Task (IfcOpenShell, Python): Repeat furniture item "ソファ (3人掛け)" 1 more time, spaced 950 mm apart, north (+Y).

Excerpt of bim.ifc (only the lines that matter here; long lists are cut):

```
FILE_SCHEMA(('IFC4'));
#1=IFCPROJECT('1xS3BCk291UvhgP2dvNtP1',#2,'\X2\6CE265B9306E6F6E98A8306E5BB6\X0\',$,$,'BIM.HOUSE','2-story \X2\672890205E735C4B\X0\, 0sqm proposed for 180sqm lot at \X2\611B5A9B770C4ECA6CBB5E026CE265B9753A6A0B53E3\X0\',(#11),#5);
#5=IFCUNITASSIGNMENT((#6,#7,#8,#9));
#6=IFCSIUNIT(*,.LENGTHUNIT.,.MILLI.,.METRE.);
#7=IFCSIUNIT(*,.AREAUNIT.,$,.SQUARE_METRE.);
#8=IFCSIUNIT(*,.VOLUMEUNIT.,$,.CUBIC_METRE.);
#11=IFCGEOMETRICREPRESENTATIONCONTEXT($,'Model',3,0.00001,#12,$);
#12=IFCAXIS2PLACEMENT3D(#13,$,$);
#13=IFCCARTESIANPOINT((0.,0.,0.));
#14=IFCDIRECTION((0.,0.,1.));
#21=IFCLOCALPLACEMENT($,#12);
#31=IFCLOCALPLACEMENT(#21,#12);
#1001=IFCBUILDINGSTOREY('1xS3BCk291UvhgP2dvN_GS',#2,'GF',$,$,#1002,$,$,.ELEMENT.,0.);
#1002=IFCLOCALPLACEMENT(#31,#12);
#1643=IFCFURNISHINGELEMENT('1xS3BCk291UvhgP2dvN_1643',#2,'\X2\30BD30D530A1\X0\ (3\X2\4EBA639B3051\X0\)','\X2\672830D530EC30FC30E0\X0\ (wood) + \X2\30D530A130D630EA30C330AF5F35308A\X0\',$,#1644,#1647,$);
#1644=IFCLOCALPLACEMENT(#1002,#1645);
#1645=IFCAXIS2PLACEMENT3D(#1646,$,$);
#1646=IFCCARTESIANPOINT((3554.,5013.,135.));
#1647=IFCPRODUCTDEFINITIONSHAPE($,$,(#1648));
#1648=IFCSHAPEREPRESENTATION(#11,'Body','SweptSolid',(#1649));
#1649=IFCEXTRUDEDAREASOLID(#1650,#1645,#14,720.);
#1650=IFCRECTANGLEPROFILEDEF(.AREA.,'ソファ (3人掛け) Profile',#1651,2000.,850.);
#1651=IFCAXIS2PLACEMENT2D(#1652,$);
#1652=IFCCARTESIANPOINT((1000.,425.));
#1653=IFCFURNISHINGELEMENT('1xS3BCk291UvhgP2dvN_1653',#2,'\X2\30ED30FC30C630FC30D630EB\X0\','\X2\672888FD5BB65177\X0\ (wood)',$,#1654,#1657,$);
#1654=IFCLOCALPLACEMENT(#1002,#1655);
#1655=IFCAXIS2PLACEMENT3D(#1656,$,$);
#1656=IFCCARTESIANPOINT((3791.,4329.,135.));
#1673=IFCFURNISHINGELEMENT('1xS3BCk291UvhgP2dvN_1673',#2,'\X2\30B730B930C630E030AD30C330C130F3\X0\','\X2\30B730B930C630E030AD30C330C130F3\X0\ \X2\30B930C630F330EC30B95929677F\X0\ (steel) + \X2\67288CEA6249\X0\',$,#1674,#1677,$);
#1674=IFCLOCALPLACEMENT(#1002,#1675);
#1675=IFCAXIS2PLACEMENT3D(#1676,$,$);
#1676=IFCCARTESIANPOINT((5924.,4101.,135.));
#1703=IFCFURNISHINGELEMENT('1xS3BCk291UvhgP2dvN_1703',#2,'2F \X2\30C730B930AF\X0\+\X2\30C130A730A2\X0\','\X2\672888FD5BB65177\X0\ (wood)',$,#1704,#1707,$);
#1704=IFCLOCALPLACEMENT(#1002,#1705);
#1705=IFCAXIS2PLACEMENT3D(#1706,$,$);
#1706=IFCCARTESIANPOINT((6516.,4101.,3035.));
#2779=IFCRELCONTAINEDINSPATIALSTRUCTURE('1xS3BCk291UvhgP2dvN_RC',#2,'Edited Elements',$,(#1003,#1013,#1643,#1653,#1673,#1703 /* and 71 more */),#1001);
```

```python
import numpy as np
import ifcopenshell
import ifcopenshell.api.geometry
import ifcopenshell.api.root
import ifcopenshell.util.element
import ifcopenshell.util.placement
import ifcopenshell.util.unit

model = ifcopenshell.open("bim.ifc")
unit_scale = ifcopenshell.util.unit.calculate_unit_scale(model)


def reuse_history(source, copy):
    """copy_class also copies each property set's owner history, people and application; keep the originals."""
    for rel in copy.IsDefinedBy:
        if rel.is_a("IfcRelDefinesByProperties") and (history := rel.RelatingPropertyDefinition.OwnerHistory):
            rel.RelatingPropertyDefinition.OwnerHistory = source.OwnerHistory
            ifcopenshell.util.element.remove_deep2(model, history)


source = model.by_id(1643)
base = ifcopenshell.util.placement.get_local_placement(source.ObjectPlacement)
step = np.array([0.0, 1.0, 0.0]) * 0.95 / unit_scale

for i in range(1, 2):
    copy = ifcopenshell.api.root.copy_class(model, product=source)
    copy.Representation = ifcopenshell.util.element.copy_deep(
        model, source.Representation, exclude=["IfcGeometricRepresentationContext", "IfcRepresentationMap"]
    )
    reuse_history(source, copy)
    matrix = base.copy()
    matrix[:3, 3] += i * step
    print("added at", matrix[:3, 3].round(3) + 0.0)
    ifcopenshell.api.geometry.edit_object_placement(model, product=copy, matrix=matrix, is_si=False)

model.write("bim_updated.ifc")
```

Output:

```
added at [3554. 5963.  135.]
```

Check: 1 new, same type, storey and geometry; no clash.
